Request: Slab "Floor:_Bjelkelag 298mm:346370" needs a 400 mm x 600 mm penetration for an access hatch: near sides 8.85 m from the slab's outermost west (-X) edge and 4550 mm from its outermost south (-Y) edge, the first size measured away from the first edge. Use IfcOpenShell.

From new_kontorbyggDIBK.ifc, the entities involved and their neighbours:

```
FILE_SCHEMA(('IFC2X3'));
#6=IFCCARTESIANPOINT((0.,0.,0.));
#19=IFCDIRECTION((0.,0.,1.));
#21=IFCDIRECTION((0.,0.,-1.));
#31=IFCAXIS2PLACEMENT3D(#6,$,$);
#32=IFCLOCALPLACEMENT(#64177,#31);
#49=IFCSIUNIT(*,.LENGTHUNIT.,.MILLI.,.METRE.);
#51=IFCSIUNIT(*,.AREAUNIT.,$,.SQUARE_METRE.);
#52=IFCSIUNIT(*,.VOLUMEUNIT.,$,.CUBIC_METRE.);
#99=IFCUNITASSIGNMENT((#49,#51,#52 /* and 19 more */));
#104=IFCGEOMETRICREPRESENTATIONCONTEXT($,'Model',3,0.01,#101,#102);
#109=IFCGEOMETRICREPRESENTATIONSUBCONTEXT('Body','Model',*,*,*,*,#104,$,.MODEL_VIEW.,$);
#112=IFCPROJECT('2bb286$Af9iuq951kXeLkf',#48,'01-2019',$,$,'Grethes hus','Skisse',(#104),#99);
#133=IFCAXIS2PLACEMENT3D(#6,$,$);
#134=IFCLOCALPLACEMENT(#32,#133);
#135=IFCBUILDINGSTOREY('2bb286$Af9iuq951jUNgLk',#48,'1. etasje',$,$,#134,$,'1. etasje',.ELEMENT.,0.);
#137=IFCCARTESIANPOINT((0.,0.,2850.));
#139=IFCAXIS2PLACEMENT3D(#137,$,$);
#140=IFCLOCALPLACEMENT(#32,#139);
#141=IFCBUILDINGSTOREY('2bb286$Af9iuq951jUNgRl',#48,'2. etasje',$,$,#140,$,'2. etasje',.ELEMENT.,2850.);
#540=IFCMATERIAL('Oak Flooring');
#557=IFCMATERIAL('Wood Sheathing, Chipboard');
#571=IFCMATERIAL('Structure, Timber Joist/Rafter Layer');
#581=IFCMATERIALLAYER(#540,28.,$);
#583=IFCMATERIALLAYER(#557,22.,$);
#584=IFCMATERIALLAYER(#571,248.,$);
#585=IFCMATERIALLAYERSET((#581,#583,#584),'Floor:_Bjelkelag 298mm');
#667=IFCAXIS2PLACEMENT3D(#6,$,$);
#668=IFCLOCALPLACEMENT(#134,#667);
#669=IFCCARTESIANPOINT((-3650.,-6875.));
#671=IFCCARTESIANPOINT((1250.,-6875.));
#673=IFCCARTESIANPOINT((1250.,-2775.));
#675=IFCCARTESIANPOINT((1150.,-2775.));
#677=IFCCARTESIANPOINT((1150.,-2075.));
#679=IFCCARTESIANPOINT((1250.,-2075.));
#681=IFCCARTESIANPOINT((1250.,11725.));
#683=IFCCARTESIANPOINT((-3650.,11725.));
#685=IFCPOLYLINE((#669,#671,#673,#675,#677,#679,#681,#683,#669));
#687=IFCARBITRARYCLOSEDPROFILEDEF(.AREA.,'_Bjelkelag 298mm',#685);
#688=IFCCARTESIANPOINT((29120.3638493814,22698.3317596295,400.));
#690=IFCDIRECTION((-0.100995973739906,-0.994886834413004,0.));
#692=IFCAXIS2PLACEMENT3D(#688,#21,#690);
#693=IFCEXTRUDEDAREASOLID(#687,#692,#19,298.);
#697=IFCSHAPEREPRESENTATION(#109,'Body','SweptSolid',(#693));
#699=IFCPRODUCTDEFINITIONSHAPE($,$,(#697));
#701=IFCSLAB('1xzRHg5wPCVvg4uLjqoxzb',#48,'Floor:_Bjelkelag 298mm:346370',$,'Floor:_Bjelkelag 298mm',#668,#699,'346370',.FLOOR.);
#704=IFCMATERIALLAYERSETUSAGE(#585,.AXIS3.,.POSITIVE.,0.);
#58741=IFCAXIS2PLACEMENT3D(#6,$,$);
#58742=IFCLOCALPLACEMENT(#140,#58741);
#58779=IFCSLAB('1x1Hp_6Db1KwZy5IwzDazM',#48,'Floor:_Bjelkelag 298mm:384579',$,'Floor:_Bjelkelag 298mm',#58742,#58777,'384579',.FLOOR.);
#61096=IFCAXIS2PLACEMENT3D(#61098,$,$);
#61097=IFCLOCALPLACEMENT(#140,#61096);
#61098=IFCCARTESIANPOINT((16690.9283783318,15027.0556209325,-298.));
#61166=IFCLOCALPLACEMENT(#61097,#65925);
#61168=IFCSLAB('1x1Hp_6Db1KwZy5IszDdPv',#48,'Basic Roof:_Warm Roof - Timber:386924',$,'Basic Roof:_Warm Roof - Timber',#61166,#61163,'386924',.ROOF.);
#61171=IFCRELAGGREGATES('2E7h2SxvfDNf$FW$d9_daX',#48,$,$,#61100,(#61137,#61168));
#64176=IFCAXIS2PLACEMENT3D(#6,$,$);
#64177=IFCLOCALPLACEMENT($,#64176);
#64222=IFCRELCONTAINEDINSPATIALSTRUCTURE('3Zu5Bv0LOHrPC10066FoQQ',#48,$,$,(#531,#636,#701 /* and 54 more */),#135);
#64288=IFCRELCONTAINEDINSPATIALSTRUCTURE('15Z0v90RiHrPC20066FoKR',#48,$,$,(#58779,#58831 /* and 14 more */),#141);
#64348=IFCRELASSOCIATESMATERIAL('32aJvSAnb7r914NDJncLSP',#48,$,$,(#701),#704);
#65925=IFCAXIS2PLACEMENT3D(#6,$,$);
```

```python
import numpy as np
import ifcopenshell
import ifcopenshell.api.feature
import ifcopenshell.api.geometry
import ifcopenshell.api.root
import ifcopenshell.geom
import ifcopenshell.util.placement
import ifcopenshell.util.representation
import ifcopenshell.util.shape
import ifcopenshell.util.unit

model = ifcopenshell.open("new_kontorbyggDIBK.ifc")
unit_scale = ifcopenshell.util.unit.calculate_unit_scale(model)
settings = ifcopenshell.geom.settings()


def volume(element):
    """Net volume in cubic metres, openings subtracted."""
    shape = ifcopenshell.geom.create_shape(settings, element)
    return ifcopenshell.util.shape.get_volume(shape.geometry)


slab = model.by_id(701)
before = volume(slab)

# Extent in the slab's own axes, in metres. The edges named are its -X and -Y sides.
slab_shape = ifcopenshell.geom.create_shape(settings, slab)
vertices = ifcopenshell.util.shape.get_vertices(slab_shape.geometry)
x_min, y_min, bottom = vertices.min(axis=0)
top = vertices[:, 2].max()

opening = ifcopenshell.api.root.create_entity(model, ifc_class="IfcOpeningElement", name="Access hatch opening")
context = ifcopenshell.util.representation.get_context(model, "Model", "Body", "MODEL_VIEW")
width, depth = 0.4, 0.6
outline = [(0.0, 0.0), (width, 0.0), (width, depth), (0.0, depth), (0.0, 0.0)]
# Overshoot both faces by 50 mm so the cut is clean.
shape = ifcopenshell.api.geometry.add_slab_representation(
    model, context=context, depth=top - bottom + 0.1, polyline=outline
)
ifcopenshell.api.geometry.assign_representation(model, product=opening, representation=shape)

matrix = ifcopenshell.util.placement.get_local_placement(slab.ObjectPlacement)
matrix[:, 3] = matrix @ np.append(np.array([x_min + 8.85, y_min + 4.55, bottom - 0.05]) / unit_scale, 1.0)
ifcopenshell.api.geometry.edit_object_placement(model, product=opening, matrix=matrix, is_si=False)
ifcopenshell.api.feature.add_feature(model, feature=opening, element=slab)

after = volume(slab)

print(f"slab volume {before:.3f} -> {after:.3f} m3")

model.write("new_kontorbyggDIBK_v2.ifc")
```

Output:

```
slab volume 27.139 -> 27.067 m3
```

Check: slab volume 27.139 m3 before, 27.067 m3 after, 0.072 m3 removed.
